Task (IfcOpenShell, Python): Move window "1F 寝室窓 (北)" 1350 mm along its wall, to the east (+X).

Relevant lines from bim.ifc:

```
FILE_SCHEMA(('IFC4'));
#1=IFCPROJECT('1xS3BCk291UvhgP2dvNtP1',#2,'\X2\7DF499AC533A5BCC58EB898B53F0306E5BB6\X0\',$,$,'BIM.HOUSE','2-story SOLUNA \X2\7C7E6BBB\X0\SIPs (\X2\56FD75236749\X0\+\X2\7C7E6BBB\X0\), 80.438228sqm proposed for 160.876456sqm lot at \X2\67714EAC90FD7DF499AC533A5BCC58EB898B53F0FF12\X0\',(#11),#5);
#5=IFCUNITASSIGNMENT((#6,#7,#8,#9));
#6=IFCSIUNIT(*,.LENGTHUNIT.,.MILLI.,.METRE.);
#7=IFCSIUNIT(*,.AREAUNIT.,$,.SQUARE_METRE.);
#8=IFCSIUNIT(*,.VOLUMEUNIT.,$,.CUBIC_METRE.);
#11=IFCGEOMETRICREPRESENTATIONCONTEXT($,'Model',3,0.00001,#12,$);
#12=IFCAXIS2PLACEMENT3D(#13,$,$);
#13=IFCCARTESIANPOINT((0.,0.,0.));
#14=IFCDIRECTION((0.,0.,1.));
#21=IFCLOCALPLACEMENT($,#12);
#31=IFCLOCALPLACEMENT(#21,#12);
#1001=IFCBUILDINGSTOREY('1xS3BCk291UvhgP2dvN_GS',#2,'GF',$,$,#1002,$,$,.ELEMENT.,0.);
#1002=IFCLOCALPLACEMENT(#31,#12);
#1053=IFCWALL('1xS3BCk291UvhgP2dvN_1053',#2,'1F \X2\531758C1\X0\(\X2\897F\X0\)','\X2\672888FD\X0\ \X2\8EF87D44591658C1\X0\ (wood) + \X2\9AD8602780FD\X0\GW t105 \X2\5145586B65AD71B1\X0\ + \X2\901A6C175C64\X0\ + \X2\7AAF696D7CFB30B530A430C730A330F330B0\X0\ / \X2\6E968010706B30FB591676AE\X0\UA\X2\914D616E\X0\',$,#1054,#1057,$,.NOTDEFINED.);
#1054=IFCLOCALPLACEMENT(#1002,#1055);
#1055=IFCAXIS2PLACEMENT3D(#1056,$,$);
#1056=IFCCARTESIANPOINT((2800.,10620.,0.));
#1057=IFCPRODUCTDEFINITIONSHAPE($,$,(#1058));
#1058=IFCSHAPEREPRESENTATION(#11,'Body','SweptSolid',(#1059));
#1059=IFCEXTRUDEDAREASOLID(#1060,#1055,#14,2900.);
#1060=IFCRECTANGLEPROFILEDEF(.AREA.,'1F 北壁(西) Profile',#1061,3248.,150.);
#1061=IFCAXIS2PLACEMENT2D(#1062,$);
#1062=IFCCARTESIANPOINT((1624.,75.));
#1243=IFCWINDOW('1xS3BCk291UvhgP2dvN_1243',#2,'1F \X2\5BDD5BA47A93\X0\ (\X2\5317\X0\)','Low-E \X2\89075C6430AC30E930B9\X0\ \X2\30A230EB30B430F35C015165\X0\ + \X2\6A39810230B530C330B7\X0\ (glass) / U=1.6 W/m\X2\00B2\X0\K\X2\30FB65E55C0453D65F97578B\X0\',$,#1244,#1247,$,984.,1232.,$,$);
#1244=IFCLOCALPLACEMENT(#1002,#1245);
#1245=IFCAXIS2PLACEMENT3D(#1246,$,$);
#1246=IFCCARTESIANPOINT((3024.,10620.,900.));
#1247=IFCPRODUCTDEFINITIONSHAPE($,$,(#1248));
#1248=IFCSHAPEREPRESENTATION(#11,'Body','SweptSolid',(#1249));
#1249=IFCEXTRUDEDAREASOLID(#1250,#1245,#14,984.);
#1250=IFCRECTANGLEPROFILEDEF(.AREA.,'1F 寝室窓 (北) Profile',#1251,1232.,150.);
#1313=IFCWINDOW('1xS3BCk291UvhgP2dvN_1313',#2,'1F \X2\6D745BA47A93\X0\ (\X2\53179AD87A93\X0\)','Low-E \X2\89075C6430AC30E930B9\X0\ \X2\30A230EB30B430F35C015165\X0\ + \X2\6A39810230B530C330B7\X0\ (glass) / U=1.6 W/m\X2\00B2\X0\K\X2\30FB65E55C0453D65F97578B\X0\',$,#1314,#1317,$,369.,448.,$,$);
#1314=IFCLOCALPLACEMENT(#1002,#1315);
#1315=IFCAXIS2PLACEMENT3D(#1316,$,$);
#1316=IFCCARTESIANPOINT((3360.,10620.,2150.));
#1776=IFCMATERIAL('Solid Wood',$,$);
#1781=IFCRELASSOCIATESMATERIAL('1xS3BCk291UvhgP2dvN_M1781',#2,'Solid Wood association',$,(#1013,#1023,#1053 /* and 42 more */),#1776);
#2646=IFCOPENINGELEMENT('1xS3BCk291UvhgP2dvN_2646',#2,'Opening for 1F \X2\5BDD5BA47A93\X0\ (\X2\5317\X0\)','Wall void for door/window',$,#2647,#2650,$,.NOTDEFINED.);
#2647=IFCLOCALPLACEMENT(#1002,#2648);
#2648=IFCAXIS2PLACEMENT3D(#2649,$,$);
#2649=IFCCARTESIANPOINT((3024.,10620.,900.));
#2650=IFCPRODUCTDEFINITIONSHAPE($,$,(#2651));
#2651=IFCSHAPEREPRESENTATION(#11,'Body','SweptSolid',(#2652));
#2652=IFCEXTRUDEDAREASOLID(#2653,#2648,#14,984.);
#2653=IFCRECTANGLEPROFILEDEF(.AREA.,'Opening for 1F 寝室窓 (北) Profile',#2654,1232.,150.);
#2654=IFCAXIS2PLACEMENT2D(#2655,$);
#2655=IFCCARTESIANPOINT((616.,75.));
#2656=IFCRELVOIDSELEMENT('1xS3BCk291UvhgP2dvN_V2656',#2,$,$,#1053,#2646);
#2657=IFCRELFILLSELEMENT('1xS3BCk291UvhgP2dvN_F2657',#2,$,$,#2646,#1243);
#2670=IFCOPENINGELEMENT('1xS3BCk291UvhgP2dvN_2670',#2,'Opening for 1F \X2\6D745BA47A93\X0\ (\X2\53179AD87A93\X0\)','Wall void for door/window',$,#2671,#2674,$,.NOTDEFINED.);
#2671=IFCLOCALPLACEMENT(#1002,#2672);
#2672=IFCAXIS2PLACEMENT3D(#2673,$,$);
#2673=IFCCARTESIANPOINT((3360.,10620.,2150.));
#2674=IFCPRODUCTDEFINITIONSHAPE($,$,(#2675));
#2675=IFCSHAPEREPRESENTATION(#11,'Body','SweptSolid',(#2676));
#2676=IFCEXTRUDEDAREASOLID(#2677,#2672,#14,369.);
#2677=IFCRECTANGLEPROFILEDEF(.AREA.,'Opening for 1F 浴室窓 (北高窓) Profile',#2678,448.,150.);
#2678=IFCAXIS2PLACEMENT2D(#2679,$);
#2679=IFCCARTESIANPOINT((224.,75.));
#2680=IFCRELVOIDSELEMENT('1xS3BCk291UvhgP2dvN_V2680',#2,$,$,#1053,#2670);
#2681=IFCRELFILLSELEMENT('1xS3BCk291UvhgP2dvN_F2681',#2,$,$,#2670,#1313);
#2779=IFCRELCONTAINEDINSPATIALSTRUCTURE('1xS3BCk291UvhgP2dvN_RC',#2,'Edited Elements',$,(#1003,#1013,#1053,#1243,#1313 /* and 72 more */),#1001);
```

```python
import ifcopenshell
import ifcopenshell.api.geometry
import ifcopenshell.util.placement
import ifcopenshell.util.unit

model = ifcopenshell.open("bim.ifc")
unit_scale = ifcopenshell.util.unit.calculate_unit_scale(model)

window = model.by_guid("1xS3BCk291UvhgP2dvN_1243")
opening = window.FillsVoids[0].RelatingOpeningElement
wall = opening.VoidsElements[0].RelatingBuildingElement

wall_matrix = ifcopenshell.util.placement.get_local_placement(wall.ObjectPlacement)
shift = wall_matrix[:3, 0] * 1.35 / unit_scale
before = ifcopenshell.util.placement.get_local_placement(window.ObjectPlacement)[:3, 3].copy()

# The window is not placed relative to its opening, so move both.
for product in (opening, window):
    matrix = ifcopenshell.util.placement.get_local_placement(product.ObjectPlacement)
    matrix[:3, 3] += shift
    ifcopenshell.api.geometry.edit_object_placement(model, product=product, matrix=matrix, is_si=False)

after = ifcopenshell.util.placement.get_local_placement(window.ObjectPlacement)[:3, 3]
print("window moved by", (after - before).round(3) + 0.0)

model.write("bim_updated.ifc")
```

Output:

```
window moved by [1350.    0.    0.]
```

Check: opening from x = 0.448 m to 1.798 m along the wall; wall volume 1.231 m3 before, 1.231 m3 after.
